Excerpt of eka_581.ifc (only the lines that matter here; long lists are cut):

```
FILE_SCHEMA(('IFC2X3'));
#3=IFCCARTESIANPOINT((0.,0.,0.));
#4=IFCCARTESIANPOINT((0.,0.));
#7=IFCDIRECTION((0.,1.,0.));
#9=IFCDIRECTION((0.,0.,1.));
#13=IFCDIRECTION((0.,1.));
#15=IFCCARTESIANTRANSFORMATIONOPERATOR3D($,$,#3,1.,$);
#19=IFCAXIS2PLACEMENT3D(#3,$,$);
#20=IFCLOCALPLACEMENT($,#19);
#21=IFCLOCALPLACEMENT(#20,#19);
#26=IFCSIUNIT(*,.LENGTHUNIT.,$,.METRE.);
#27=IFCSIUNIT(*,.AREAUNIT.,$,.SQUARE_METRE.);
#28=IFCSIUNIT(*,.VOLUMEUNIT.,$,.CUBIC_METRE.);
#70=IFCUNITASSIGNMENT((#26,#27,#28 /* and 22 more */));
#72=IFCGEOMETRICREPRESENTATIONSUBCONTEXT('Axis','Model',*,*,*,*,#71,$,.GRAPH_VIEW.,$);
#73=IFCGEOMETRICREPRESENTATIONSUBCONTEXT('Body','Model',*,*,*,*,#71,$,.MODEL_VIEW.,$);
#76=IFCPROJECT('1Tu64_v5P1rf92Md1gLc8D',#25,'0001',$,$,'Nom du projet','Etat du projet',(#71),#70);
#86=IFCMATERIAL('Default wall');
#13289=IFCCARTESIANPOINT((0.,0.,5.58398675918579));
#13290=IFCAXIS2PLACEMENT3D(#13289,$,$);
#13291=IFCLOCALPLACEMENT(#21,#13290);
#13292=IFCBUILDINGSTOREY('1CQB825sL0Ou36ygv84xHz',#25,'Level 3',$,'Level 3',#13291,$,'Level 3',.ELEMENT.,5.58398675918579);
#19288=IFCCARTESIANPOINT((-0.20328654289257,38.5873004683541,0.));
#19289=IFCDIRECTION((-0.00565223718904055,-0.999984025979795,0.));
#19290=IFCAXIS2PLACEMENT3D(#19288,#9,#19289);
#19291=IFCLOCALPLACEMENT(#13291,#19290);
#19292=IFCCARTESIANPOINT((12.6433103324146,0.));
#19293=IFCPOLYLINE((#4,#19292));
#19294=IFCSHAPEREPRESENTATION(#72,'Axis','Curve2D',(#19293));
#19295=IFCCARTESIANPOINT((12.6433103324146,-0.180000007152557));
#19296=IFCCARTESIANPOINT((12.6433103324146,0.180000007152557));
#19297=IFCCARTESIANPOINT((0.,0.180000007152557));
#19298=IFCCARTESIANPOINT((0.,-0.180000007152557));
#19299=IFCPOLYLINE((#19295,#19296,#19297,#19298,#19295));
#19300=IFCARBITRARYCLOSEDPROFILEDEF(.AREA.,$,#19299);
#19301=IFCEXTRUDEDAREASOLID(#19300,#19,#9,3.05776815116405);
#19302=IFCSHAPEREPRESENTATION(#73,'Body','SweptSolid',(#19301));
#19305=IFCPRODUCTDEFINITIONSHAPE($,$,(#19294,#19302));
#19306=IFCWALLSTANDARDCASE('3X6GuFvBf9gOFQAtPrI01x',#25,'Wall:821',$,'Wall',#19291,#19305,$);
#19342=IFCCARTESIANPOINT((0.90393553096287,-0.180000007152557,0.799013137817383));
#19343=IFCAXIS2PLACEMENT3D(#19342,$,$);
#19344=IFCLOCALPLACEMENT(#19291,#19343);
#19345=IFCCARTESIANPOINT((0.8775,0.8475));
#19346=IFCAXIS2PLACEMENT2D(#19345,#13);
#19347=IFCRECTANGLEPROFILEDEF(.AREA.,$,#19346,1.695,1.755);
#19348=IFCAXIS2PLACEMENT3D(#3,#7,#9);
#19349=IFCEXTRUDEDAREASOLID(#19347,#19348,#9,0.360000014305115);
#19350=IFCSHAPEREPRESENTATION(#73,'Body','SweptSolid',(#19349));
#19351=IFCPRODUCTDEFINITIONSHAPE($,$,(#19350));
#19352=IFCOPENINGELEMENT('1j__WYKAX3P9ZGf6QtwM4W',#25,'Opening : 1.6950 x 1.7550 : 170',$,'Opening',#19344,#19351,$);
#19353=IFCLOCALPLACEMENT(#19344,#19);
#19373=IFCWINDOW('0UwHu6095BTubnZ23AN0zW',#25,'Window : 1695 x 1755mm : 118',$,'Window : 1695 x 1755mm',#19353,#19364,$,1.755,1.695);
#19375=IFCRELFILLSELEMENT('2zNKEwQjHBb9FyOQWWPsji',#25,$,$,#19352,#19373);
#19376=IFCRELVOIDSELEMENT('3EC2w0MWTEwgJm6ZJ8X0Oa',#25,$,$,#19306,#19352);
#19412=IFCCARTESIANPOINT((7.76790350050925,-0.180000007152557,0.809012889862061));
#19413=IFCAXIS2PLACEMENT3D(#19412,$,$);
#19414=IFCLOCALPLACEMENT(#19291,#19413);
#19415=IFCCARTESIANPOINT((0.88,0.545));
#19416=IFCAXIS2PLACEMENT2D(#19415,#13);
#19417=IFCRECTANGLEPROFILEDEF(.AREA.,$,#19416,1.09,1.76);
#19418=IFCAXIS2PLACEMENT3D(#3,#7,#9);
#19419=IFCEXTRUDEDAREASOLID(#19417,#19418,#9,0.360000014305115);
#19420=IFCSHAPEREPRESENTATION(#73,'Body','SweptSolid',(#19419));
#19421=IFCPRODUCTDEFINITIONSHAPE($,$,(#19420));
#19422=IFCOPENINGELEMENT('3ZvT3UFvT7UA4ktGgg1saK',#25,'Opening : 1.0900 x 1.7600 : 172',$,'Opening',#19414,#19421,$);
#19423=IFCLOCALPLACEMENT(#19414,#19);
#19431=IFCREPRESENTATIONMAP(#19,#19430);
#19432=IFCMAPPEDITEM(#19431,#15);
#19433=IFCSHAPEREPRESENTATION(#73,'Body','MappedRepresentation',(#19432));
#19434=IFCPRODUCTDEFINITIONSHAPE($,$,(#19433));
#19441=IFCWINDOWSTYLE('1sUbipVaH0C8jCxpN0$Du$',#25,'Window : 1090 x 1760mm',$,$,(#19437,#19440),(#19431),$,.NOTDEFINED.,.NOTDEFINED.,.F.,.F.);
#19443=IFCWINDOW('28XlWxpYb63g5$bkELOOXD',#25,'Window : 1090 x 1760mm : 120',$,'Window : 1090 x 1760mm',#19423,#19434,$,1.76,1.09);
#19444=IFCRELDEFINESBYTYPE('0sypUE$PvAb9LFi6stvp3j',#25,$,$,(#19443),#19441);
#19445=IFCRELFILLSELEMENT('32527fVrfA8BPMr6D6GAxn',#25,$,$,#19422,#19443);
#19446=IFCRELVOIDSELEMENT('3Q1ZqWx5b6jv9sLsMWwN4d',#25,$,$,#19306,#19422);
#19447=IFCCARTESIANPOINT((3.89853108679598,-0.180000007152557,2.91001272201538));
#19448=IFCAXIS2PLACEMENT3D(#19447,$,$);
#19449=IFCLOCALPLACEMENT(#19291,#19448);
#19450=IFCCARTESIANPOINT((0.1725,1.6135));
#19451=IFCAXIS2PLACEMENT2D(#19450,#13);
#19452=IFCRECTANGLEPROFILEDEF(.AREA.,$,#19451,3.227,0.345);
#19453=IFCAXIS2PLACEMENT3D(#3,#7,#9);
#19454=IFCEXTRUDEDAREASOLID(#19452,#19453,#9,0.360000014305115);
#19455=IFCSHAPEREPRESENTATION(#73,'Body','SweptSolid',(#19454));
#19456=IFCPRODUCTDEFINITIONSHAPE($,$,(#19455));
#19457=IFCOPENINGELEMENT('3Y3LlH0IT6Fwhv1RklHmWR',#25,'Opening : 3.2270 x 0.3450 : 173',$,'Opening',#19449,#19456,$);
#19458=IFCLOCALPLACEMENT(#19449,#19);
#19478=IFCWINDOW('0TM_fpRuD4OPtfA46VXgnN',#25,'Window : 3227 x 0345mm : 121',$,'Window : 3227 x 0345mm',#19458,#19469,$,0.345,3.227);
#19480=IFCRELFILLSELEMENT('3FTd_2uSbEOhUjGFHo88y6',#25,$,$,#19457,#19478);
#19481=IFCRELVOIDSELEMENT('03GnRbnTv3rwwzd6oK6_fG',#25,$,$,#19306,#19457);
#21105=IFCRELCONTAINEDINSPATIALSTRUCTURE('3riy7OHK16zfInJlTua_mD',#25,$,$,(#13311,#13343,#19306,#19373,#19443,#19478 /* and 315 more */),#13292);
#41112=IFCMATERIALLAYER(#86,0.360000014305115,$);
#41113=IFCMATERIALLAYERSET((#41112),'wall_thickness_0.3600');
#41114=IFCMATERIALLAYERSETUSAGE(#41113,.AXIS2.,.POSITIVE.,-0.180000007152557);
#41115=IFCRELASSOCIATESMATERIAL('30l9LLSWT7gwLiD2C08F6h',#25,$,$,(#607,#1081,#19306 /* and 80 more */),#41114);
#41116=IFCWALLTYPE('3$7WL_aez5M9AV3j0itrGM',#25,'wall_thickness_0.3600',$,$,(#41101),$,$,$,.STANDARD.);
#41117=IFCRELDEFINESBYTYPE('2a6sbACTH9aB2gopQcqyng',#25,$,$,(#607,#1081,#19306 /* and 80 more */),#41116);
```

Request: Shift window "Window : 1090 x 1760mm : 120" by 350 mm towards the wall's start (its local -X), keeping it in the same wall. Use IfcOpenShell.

```python
import ifcopenshell
import ifcopenshell.api.geometry
import ifcopenshell.util.placement
import ifcopenshell.util.unit

model = ifcopenshell.open("eka_581.ifc")
unit_scale = ifcopenshell.util.unit.calculate_unit_scale(model)

window = model.by_id(19443)
opening = window.FillsVoids[0].RelatingOpeningElement
wall = opening.VoidsElements[0].RelatingBuildingElement

wall_matrix = ifcopenshell.util.placement.get_local_placement(wall.ObjectPlacement)
shift = wall_matrix[:3, 0] * -0.35 / unit_scale
before = ifcopenshell.util.placement.get_local_placement(window.ObjectPlacement)[:3, 3].copy()

# The window is placed relative to its opening, so it follows when the opening moves.
matrix = ifcopenshell.util.placement.get_local_placement(opening.ObjectPlacement)
matrix[:3, 3] += shift
ifcopenshell.api.geometry.edit_object_placement(
    model, product=opening, matrix=matrix, is_si=False, should_transform_children=True
)

after = ifcopenshell.util.placement.get_local_placement(window.ObjectPlacement)[:3, 3]
print("window moved by", (after - before).round(3) + 0.0)

model.write("eka_581-out.ifc")
```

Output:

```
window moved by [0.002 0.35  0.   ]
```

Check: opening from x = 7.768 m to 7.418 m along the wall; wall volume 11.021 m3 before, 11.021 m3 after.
